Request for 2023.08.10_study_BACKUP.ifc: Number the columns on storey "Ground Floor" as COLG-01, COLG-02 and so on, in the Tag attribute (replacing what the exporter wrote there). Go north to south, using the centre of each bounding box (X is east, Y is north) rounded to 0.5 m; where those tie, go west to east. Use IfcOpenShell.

First a look at what the model holds.

```python
import ifcopenshell
import ifcopenshell.util.element
import ifcopenshell.util.placement

model = ifcopenshell.open("2023.08.10_study_BACKUP.ifc")
print(model.schema)
storey = next(s for s in model.by_type("IfcBuildingStorey") if s.Name == "Ground Floor")
columns = [e for e in ifcopenshell.util.element.get_decomposition(storey) if e.is_a("IfcColumn")]
for e in sorted(columns, key=lambda e: e.id()):
    origin = ifcopenshell.util.placement.get_local_placement(e.ObjectPlacement)[:3, 3]
    print(e.id(), e.Tag, e.Name, origin.round(2) + 0.0, sep=" | ")
```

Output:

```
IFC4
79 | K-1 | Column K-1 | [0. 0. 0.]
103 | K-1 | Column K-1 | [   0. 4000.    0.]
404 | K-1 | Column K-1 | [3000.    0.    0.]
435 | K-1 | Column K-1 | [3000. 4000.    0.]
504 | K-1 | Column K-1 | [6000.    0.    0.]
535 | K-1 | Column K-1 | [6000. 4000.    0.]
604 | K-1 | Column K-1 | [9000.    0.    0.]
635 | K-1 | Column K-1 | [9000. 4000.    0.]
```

```python
import ifcopenshell
import ifcopenshell.geom
import ifcopenshell.util.element
import ifcopenshell.util.shape

model = ifcopenshell.open("2023.08.10_study_BACKUP.ifc")
settings = ifcopenshell.geom.settings()
settings.set("use-world-coords", True)


def centre(element):
    shape = ifcopenshell.geom.create_shape(settings, element)
    return ifcopenshell.util.shape.get_bbox_centroid(shape.geometry)


storey = next(s for s in model.by_type("IfcBuildingStorey") if s.Name == "Ground Floor")
columns = [e for e in ifcopenshell.util.element.get_decomposition(storey) if e.is_a("IfcColumn")]

# Insertion points can sit at a corner or the storey origin, so sort by the geometry (in metres).
centres = {e: centre(e) for e in columns}
columns.sort(key=lambda e: (-round(centres[e][1] / 0.5), centres[e][0]))

for i, e in enumerate(columns, start=1):
    number = f"COLG-{i:02d}"
    e.Tag = number
    print(e.id(), number)

model.write("2023.08.10_study_BACKUP-out.ifc")
```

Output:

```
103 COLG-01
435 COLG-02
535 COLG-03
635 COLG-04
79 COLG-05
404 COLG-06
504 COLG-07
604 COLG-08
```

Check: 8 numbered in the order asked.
